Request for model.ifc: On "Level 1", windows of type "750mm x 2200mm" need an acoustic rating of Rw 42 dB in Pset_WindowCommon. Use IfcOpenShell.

First a look at what the model holds.

```python
import ifcopenshell
import ifcopenshell.util.element

model = ifcopenshell.open("model.ifc")
print(model.schema)
storey = next(s for s in model.by_type("IfcBuildingStorey") if s.Name == "Level 1")
windows = [e for e in ifcopenshell.util.element.get_decomposition(storey) if e.is_a("IfcWindow")]
seen = {}
for e in windows:
    element_type = ifcopenshell.util.element.get_type(e)
    key = (element_type.Name if element_type != e and element_type else None, ifcopenshell.util.element.get_pset(e, "Pset_WindowCommon", "AcousticRating"))
    seen[key] = seen.get(key, 0) + 1
for (name, value), count in sorted(seen.items(), key=str):
    print(count, "x", name, "|", value)
```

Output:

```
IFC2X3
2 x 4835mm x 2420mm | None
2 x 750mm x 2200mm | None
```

```python
import ifcopenshell
import ifcopenshell.api.pset
import ifcopenshell.util.element

model = ifcopenshell.open("model.ifc")

storey = next(s for s in model.by_type("IfcBuildingStorey") if s.Name == "Level 1")
windows = [e for e in ifcopenshell.util.element.get_decomposition(storey) if e.is_a("IfcWindow")]

count = 0
for e in windows:
    element_type = ifcopenshell.util.element.get_type(e)
    if element_type in (None, e) or element_type.Name != "750mm x 2200mm":
        continue
    # add_pset returns the element's existing set when there is one.
    pset = ifcopenshell.api.pset.add_pset(model, product=e, name="Pset_WindowCommon")
    ifcopenshell.api.pset.edit_pset(model, pset=pset, properties={"AcousticRating": "Rw 42 dB"})
    count += 1

print(count, "windows updated")

model.write("model_v2.ifc")
```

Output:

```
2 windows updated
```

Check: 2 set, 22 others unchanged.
